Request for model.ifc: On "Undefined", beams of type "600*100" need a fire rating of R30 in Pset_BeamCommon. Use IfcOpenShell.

First a look at what the model holds.

```python
import ifcopenshell
import ifcopenshell.util.element

model = ifcopenshell.open("model.ifc")
print(model.schema)
storey = next(s for s in model.by_type("IfcBuildingStorey") if s.Name == "Undefined")
beams = [e for e in ifcopenshell.util.element.get_decomposition(storey) if e.is_a("IfcBeam")]
seen = {}
for e in beams:
    element_type = ifcopenshell.util.element.get_type(e)
    key = (element_type.Name if element_type != e and element_type else None, ifcopenshell.util.element.get_pset(e, "Pset_BeamCommon", "FireRating"))
    seen[key] = seen.get(key, 0) + 1
for (name, value), count in sorted(seen.items(), key=str):
    print(count, "x", name, "|", value)
```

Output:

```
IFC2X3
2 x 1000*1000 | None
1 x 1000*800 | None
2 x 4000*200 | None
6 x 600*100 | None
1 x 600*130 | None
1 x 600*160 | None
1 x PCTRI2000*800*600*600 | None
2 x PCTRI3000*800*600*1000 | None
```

```python
import ifcopenshell
import ifcopenshell.api.pset
import ifcopenshell.util.element

model = ifcopenshell.open("model.ifc")

storey = next(s for s in model.by_type("IfcBuildingStorey") if s.Name == "Undefined")
beams = [e for e in ifcopenshell.util.element.get_decomposition(storey) if e.is_a("IfcBeam")]

count = 0
for e in beams:
    element_type = ifcopenshell.util.element.get_type(e)
    if element_type in (None, e) or element_type.Name != "600*100":
        continue
    found = ifcopenshell.util.element.get_pset(e, "Pset_BeamCommon", should_inherit=False)
    if found:
        pset = model.by_id(found["id"])
        if len(ifcopenshell.util.element.get_elements_by_pset(pset)) > 1:
            pset = ifcopenshell.api.pset.unshare_pset(model, products=[e], pset=pset)[0]
    else:
        pset = ifcopenshell.api.pset.add_pset(model, product=e, name="Pset_BeamCommon")
    ifcopenshell.api.pset.edit_pset(model, pset=pset, properties={"FireRating": "R30"})
    count += 1

print(count, "beams updated")

model.write("model_edited.ifc")
```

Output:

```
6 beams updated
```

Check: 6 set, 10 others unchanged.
